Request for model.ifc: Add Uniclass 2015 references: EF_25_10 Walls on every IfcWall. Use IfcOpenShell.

First a look at what the model holds.

```python
import ifcopenshell

model = ifcopenshell.open("model.ifc")
print(model.schema)
print("classifications:", [c.Name for c in model.by_type("IfcClassification")])
for ifc_class in ("IfcDoor", "IfcRoof", "IfcStair", "IfcWall", "IfcWindow"):
    print(ifc_class, len(model.by_type(ifc_class)))
```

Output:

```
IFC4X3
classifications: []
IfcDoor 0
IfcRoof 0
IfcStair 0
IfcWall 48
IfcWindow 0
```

```python
import ifcopenshell
import ifcopenshell.api.classification

model = ifcopenshell.open("model.ifc")

system = ifcopenshell.api.classification.add_classification(model, classification="Uniclass 2015")

codes = {
    "IfcWall": ("EF_25_10", "Walls"),
}
for ifc_class, (code, name) in codes.items():
    products = model.by_type(ifc_class)
    ifcopenshell.api.classification.add_reference(
        model, products=products, classification=system, identification=code, name=name
    )
    print(code, len(products))

model.write("model-out.ifc")
```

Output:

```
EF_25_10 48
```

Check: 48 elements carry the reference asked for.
